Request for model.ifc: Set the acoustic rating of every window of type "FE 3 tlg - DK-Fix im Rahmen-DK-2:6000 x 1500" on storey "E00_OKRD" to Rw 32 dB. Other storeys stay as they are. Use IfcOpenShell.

First a look at what the model holds.

```python
import ifcopenshell
import ifcopenshell.util.element

model = ifcopenshell.open("model.ifc")
print(model.schema)
storey = next(s for s in model.by_type("IfcBuildingStorey") if s.Name == "E00_OKRD")
windows = [e for e in ifcopenshell.util.element.get_decomposition(storey) if e.is_a("IfcWindow")]
seen = {}
for e in windows:
    element_type = ifcopenshell.util.element.get_type(e)
    key = (element_type.Name if element_type != e and element_type else None, ifcopenshell.util.element.get_pset(e, "Pset_WindowCommon", "AcousticRating"))
    seen[key] = seen.get(key, 0) + 1
for (name, value), count in sorted(seen.items(), key=str):
    print(count, "x", name, "|", value)
```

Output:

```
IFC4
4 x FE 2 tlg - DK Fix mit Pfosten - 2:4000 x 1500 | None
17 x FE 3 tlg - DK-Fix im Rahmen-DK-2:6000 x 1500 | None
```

```python
import ifcopenshell
import ifcopenshell.api.pset
import ifcopenshell.util.element

model = ifcopenshell.open("model.ifc")

storey = next(s for s in model.by_type("IfcBuildingStorey") if s.Name == "E00_OKRD")
windows = [e for e in ifcopenshell.util.element.get_decomposition(storey) if e.is_a("IfcWindow")]

count = 0
for e in windows:
    element_type = ifcopenshell.util.element.get_type(e)
    if element_type in (None, e) or element_type.Name != "FE 3 tlg - DK-Fix im Rahmen-DK-2:6000 x 1500":
        continue
    # add_pset returns the element's existing set when there is one.
    pset = ifcopenshell.api.pset.add_pset(model, product=e, name="Pset_WindowCommon")
    ifcopenshell.api.pset.edit_pset(model, pset=pset, properties={"AcousticRating": "Rw 32 dB"})
    count += 1

print(count, "windows updated")

model.write("model_updated.ifc")
```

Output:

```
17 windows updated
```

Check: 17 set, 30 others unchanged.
